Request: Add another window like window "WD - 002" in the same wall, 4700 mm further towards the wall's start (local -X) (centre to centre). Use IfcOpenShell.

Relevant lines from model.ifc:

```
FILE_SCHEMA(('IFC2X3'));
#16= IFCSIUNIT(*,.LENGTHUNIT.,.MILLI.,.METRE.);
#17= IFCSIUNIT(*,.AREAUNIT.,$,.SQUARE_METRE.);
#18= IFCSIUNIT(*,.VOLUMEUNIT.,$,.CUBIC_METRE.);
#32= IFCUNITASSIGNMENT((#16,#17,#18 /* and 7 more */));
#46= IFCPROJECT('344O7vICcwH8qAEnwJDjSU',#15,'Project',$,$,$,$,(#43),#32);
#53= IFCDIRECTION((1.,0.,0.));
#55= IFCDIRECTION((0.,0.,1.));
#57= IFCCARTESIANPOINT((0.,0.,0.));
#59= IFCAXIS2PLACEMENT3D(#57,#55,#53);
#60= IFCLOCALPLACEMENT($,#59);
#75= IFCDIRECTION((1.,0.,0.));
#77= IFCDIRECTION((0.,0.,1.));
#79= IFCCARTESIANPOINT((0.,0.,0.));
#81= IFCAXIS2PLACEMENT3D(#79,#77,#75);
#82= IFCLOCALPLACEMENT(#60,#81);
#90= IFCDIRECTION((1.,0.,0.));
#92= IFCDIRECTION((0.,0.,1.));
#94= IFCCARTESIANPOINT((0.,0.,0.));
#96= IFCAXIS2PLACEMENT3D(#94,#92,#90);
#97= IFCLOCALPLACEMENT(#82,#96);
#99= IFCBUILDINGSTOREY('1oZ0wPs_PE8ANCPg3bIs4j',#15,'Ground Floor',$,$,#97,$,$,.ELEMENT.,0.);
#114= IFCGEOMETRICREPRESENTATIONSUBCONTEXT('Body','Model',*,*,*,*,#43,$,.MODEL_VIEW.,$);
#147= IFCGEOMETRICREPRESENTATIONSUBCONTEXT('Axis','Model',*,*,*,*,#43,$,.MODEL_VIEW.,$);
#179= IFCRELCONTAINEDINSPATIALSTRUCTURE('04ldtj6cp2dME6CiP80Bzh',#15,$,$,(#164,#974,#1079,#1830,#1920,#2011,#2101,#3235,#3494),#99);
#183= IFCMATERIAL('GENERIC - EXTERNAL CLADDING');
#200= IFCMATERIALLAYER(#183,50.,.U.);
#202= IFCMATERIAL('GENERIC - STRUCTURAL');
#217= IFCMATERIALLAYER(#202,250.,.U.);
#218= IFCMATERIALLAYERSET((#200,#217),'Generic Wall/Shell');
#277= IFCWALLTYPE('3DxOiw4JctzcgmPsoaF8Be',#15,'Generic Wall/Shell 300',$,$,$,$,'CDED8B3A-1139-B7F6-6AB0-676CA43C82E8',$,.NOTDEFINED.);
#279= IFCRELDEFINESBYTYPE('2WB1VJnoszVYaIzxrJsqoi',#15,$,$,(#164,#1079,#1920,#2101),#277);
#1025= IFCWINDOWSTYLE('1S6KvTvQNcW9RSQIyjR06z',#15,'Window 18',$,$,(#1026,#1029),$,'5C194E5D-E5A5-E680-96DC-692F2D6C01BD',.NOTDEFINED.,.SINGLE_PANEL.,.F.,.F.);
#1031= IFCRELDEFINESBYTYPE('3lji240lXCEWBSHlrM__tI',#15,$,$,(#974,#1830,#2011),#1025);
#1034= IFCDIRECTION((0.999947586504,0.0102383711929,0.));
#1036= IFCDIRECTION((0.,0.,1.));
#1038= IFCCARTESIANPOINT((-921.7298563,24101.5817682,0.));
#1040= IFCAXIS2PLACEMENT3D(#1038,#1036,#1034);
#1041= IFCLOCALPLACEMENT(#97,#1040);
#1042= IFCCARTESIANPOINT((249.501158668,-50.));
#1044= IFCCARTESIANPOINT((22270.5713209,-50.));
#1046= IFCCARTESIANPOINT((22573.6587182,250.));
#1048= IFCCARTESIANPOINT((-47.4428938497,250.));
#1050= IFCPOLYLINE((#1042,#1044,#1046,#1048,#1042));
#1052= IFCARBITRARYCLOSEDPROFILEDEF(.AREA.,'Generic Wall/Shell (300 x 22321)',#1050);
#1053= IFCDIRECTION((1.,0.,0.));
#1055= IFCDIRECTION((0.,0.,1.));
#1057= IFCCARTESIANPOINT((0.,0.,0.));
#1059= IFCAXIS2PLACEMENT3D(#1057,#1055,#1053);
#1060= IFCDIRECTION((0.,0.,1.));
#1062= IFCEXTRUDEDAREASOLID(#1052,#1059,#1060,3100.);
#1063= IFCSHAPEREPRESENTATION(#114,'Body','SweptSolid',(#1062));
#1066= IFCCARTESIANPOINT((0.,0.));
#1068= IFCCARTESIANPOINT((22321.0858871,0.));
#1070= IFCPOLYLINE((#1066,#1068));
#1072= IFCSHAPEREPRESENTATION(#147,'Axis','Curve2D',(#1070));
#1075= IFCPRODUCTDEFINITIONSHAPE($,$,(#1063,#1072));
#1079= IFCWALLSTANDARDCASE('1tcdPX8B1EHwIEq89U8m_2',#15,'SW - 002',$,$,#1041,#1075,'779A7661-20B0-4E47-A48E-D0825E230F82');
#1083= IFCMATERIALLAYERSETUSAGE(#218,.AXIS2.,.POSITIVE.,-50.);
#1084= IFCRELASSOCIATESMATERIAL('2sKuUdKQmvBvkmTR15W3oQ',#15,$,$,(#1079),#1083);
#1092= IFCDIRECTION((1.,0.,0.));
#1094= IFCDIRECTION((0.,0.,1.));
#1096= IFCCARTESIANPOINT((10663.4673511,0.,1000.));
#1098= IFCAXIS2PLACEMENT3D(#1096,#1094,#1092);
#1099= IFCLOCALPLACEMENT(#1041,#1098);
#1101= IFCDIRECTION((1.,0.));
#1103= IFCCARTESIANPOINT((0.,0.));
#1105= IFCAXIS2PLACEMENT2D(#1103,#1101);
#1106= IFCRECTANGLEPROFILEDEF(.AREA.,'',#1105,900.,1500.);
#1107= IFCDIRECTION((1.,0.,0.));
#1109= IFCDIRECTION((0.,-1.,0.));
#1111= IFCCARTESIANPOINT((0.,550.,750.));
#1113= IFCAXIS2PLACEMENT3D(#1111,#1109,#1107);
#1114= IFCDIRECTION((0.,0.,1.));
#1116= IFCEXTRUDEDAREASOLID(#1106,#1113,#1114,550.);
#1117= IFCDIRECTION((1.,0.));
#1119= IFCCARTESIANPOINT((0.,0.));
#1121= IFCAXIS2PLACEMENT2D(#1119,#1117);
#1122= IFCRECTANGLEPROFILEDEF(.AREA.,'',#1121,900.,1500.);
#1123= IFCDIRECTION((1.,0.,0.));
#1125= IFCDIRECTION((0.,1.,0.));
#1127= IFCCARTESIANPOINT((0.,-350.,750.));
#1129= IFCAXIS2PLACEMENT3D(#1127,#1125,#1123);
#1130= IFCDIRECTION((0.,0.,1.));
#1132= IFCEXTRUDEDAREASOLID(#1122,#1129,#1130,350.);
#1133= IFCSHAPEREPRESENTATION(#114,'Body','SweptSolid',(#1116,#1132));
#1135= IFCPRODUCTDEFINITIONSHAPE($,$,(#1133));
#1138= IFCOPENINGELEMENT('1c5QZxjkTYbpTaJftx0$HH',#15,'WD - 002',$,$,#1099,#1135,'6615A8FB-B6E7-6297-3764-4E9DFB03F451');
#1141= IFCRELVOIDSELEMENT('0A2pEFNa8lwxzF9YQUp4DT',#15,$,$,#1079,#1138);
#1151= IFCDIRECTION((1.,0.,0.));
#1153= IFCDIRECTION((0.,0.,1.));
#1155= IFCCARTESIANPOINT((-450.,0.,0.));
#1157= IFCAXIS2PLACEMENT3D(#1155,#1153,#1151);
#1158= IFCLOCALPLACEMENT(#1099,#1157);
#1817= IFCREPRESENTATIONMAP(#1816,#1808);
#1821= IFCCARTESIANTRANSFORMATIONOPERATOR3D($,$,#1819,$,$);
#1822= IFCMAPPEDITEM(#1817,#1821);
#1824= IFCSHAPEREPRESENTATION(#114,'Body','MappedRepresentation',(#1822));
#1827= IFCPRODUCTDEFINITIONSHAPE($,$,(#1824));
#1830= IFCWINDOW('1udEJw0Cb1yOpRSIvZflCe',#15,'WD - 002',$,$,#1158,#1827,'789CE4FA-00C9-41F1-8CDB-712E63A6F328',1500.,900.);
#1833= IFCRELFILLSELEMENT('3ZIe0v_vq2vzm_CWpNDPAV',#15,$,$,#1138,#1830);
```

```python
import ifcopenshell
import ifcopenshell.api.feature
import ifcopenshell.api.geometry
import ifcopenshell.api.root
import ifcopenshell.geom
import ifcopenshell.util.element
import ifcopenshell.util.placement
import ifcopenshell.util.shape
import ifcopenshell.util.unit

model = ifcopenshell.open("model.ifc")
unit_scale = ifcopenshell.util.unit.calculate_unit_scale(model)
settings = ifcopenshell.geom.settings()


def volume(element):
    """Net volume in cubic metres, openings subtracted."""
    shape = ifcopenshell.geom.create_shape(settings, element)
    return ifcopenshell.util.shape.get_volume(shape.geometry)


def reuse_history(source, copy):
    """copy_class also copies each property set's owner history, people and application; keep the originals."""
    for rel in copy.IsDefinedBy:
        if rel.is_a("IfcRelDefinesByProperties") and (history := rel.RelatingPropertyDefinition.OwnerHistory):
            rel.RelatingPropertyDefinition.OwnerHistory = source.OwnerHistory
            ifcopenshell.util.element.remove_deep2(model, history)


window = model.by_guid("1udEJw0Cb1yOpRSIvZflCe")
opening = window.FillsVoids[0].RelatingOpeningElement
wall = opening.VoidsElements[0].RelatingBuildingElement
before = volume(wall)
shift = ifcopenshell.util.placement.get_local_placement(wall.ObjectPlacement)[:3, 0] * -4.7 / unit_scale

# copy_class copies the void relationship, type, container and properties, but no geometry.
new_opening = ifcopenshell.api.root.copy_class(model, product=opening)
new_opening.Representation = ifcopenshell.util.element.copy_deep(
    model, opening.Representation, exclude=["IfcGeometricRepresentationContext", "IfcRepresentationMap"]
)
new_opening.Tag = None
new_window = ifcopenshell.api.root.copy_class(model, product=window)
new_window.Representation = ifcopenshell.util.element.copy_deep(
    model, window.Representation, exclude=["IfcGeometricRepresentationContext", "IfcRepresentationMap"]
)
new_window.Tag = None
reuse_history(window, new_window)
fills = ifcopenshell.api.feature.add_filling(model, opening=new_opening, element=new_window)
fills.OwnerHistory = new_window.OwnerHistory  # required in IFC2X3

for old, new in ((opening, new_opening), (window, new_window)):
    matrix = ifcopenshell.util.placement.get_local_placement(old.ObjectPlacement)
    matrix[:3, 3] += shift
    ifcopenshell.api.geometry.edit_object_placement(model, product=new, matrix=matrix, is_si=False)

after = volume(wall)

print(f"wall volume {before:.3f} -> {after:.3f} m3")

model.write("model-out.ifc")
```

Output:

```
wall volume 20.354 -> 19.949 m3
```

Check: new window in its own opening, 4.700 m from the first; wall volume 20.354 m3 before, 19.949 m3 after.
